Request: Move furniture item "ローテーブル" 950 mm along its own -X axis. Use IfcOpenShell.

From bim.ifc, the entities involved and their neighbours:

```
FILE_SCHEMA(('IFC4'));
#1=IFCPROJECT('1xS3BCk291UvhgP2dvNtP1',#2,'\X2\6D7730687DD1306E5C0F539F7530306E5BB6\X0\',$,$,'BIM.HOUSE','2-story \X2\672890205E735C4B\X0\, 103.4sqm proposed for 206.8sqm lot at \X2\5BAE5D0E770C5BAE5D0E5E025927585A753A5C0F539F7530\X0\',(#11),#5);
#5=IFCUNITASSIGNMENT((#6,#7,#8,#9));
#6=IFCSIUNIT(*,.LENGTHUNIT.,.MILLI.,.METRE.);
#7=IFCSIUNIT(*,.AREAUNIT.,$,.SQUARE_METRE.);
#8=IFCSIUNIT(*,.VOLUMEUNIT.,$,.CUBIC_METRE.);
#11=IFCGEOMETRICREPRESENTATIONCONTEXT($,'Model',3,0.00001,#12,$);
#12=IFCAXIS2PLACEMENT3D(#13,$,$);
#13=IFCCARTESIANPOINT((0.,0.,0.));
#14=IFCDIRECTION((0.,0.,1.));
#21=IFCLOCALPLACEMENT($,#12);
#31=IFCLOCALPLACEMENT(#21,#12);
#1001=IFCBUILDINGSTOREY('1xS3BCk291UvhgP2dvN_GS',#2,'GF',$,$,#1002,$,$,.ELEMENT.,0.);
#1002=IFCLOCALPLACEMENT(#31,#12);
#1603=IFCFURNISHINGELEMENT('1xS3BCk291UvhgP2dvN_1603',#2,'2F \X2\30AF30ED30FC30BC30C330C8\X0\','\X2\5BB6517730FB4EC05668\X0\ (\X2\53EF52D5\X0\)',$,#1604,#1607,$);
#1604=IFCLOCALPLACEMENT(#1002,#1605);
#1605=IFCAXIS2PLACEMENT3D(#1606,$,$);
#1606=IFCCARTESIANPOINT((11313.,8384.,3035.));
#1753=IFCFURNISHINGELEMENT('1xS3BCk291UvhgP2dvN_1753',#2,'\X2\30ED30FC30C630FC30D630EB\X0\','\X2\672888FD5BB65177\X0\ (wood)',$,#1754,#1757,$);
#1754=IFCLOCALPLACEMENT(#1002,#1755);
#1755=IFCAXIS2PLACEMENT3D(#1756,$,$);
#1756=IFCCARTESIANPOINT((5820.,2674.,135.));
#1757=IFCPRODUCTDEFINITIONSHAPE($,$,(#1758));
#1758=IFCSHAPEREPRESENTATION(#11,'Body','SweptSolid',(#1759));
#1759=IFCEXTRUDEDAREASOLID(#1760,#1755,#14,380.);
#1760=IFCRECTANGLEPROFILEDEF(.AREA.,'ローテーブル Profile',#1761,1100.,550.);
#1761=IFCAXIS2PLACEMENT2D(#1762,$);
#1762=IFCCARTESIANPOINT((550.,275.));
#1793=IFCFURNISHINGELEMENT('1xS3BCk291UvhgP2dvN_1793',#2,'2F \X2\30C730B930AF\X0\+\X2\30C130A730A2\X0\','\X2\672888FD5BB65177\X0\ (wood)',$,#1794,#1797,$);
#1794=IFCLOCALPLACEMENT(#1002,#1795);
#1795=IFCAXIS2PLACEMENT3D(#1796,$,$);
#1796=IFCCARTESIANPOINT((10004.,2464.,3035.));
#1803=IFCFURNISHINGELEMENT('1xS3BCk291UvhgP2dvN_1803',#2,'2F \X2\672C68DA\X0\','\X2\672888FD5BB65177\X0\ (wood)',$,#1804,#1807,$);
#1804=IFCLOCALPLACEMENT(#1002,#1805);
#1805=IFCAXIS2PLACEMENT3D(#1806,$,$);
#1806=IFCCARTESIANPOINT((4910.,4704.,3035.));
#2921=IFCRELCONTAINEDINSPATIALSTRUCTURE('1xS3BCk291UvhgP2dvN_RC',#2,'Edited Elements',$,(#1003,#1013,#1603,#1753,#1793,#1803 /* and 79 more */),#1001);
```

```python
import ifcopenshell
import ifcopenshell.api.geometry
import ifcopenshell.util.placement

model = ifcopenshell.open("bim.ifc")

item = model.by_guid("1xS3BCk291UvhgP2dvN_1753")
matrix = ifcopenshell.util.placement.get_local_placement(item.ObjectPlacement)
matrix[:3, 3] -= matrix[:3, 0] * 950.0
ifcopenshell.api.geometry.edit_object_placement(model, product=item, matrix=matrix, is_si=False)

print(ifcopenshell.util.placement.get_local_placement(item.ObjectPlacement).round(3) + 0.0)

model.write("bim_v2.ifc")
```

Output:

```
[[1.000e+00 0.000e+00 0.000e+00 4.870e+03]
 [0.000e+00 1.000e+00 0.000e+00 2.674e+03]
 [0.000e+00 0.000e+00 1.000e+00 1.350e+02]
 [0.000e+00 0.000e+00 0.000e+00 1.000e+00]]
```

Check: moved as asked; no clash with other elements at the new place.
